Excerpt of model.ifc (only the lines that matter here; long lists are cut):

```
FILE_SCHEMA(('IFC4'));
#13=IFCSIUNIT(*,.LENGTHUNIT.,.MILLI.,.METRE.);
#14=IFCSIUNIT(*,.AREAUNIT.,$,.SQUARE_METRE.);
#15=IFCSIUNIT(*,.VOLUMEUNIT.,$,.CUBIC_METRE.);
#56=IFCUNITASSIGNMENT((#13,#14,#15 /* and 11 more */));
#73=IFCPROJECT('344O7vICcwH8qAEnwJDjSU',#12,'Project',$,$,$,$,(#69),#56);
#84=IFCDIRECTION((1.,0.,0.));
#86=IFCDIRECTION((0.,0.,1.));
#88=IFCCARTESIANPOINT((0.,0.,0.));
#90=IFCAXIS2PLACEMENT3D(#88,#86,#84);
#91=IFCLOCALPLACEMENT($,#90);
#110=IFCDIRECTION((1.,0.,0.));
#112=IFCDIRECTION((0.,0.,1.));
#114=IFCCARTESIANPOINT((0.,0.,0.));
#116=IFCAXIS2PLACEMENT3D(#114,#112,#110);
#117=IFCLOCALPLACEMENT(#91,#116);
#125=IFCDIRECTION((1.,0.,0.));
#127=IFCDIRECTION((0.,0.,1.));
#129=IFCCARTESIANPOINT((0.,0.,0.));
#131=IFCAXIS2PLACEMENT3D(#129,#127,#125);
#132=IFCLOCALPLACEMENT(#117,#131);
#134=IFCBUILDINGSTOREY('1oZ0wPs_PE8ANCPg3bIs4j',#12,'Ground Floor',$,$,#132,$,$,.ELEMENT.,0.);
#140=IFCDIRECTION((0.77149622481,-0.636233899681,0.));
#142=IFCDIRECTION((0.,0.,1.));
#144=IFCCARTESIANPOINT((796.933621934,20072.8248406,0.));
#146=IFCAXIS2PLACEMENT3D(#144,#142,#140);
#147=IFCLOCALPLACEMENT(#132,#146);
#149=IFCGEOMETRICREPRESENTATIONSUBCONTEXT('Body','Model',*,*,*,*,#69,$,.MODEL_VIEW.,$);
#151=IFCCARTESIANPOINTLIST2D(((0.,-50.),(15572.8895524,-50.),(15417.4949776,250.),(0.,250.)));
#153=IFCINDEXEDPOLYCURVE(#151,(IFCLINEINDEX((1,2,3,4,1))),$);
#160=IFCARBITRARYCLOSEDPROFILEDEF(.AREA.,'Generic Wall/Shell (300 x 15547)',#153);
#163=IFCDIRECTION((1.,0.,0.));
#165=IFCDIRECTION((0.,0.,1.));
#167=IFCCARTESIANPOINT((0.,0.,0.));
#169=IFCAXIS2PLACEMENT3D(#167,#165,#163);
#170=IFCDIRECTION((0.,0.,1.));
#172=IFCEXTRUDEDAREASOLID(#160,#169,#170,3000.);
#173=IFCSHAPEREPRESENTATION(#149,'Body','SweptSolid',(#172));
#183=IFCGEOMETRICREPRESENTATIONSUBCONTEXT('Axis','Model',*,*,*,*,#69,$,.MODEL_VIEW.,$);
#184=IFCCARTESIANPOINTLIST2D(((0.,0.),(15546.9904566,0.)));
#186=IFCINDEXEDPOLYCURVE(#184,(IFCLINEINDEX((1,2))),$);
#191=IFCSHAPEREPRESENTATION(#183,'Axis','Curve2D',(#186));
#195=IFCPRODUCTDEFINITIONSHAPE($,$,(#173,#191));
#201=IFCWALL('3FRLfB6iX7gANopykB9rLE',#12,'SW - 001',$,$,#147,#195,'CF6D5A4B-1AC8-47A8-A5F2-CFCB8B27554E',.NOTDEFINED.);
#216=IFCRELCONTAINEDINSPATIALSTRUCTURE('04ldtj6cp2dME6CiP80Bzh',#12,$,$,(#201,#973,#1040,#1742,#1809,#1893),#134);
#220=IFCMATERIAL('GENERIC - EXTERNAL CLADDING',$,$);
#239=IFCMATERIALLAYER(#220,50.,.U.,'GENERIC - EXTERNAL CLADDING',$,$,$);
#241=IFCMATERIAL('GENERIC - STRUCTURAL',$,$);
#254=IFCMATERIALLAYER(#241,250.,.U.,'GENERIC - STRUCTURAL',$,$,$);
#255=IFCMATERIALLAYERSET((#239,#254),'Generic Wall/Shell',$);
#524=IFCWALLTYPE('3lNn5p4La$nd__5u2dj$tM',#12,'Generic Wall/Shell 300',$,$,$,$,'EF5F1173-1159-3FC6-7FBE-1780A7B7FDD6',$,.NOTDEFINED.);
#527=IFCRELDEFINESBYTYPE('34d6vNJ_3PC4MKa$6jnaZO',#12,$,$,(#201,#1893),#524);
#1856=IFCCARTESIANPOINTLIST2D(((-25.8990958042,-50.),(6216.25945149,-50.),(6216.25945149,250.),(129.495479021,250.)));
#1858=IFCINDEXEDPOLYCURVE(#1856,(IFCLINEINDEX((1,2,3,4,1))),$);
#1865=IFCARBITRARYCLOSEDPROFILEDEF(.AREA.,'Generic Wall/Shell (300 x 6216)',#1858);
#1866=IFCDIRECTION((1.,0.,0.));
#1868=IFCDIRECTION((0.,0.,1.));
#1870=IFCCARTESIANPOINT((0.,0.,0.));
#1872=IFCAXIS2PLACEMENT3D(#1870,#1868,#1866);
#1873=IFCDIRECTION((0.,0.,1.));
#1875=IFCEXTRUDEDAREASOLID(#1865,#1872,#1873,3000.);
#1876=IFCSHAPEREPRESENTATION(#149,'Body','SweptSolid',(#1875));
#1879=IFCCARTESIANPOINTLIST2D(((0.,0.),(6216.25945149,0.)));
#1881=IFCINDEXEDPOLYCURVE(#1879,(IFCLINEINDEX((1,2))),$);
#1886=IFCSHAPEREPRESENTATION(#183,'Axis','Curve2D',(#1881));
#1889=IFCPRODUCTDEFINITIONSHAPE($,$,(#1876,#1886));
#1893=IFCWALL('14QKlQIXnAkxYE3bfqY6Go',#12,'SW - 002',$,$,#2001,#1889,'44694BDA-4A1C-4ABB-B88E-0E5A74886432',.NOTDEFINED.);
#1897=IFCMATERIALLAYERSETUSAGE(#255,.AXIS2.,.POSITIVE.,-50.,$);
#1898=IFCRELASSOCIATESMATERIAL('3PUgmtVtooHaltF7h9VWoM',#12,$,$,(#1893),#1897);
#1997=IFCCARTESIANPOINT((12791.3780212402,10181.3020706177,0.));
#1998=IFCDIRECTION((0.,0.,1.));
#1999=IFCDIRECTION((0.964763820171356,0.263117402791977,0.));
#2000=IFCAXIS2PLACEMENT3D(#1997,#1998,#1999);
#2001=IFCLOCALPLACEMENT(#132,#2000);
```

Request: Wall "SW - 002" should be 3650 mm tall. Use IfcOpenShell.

```python
import ifcopenshell
import ifcopenshell.geom
import ifcopenshell.util.representation
import ifcopenshell.util.shape
import ifcopenshell.util.unit

model = ifcopenshell.open("model.ifc")
unit_scale = ifcopenshell.util.unit.calculate_unit_scale(model)
settings = ifcopenshell.geom.settings()


def volume(element):
    """Net volume in cubic metres, openings subtracted."""
    shape = ifcopenshell.geom.create_shape(settings, element)
    return ifcopenshell.util.shape.get_volume(shape.geometry)


wall = model.by_id(1893)
before = volume(wall)

body = ifcopenshell.util.representation.get_representation(wall, "Model", "Body")
solid = body.Items[0]
old_height = solid.Depth
solid.Depth = 3.65 / unit_scale
after = volume(wall)

print(f"height {old_height:g} -> {solid.Depth:g}, volume {before:.3f} -> {after:.3f} m3")

model.write("model_updated.ifc")
```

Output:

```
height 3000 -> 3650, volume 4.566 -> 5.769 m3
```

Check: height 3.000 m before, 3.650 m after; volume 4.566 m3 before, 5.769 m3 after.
